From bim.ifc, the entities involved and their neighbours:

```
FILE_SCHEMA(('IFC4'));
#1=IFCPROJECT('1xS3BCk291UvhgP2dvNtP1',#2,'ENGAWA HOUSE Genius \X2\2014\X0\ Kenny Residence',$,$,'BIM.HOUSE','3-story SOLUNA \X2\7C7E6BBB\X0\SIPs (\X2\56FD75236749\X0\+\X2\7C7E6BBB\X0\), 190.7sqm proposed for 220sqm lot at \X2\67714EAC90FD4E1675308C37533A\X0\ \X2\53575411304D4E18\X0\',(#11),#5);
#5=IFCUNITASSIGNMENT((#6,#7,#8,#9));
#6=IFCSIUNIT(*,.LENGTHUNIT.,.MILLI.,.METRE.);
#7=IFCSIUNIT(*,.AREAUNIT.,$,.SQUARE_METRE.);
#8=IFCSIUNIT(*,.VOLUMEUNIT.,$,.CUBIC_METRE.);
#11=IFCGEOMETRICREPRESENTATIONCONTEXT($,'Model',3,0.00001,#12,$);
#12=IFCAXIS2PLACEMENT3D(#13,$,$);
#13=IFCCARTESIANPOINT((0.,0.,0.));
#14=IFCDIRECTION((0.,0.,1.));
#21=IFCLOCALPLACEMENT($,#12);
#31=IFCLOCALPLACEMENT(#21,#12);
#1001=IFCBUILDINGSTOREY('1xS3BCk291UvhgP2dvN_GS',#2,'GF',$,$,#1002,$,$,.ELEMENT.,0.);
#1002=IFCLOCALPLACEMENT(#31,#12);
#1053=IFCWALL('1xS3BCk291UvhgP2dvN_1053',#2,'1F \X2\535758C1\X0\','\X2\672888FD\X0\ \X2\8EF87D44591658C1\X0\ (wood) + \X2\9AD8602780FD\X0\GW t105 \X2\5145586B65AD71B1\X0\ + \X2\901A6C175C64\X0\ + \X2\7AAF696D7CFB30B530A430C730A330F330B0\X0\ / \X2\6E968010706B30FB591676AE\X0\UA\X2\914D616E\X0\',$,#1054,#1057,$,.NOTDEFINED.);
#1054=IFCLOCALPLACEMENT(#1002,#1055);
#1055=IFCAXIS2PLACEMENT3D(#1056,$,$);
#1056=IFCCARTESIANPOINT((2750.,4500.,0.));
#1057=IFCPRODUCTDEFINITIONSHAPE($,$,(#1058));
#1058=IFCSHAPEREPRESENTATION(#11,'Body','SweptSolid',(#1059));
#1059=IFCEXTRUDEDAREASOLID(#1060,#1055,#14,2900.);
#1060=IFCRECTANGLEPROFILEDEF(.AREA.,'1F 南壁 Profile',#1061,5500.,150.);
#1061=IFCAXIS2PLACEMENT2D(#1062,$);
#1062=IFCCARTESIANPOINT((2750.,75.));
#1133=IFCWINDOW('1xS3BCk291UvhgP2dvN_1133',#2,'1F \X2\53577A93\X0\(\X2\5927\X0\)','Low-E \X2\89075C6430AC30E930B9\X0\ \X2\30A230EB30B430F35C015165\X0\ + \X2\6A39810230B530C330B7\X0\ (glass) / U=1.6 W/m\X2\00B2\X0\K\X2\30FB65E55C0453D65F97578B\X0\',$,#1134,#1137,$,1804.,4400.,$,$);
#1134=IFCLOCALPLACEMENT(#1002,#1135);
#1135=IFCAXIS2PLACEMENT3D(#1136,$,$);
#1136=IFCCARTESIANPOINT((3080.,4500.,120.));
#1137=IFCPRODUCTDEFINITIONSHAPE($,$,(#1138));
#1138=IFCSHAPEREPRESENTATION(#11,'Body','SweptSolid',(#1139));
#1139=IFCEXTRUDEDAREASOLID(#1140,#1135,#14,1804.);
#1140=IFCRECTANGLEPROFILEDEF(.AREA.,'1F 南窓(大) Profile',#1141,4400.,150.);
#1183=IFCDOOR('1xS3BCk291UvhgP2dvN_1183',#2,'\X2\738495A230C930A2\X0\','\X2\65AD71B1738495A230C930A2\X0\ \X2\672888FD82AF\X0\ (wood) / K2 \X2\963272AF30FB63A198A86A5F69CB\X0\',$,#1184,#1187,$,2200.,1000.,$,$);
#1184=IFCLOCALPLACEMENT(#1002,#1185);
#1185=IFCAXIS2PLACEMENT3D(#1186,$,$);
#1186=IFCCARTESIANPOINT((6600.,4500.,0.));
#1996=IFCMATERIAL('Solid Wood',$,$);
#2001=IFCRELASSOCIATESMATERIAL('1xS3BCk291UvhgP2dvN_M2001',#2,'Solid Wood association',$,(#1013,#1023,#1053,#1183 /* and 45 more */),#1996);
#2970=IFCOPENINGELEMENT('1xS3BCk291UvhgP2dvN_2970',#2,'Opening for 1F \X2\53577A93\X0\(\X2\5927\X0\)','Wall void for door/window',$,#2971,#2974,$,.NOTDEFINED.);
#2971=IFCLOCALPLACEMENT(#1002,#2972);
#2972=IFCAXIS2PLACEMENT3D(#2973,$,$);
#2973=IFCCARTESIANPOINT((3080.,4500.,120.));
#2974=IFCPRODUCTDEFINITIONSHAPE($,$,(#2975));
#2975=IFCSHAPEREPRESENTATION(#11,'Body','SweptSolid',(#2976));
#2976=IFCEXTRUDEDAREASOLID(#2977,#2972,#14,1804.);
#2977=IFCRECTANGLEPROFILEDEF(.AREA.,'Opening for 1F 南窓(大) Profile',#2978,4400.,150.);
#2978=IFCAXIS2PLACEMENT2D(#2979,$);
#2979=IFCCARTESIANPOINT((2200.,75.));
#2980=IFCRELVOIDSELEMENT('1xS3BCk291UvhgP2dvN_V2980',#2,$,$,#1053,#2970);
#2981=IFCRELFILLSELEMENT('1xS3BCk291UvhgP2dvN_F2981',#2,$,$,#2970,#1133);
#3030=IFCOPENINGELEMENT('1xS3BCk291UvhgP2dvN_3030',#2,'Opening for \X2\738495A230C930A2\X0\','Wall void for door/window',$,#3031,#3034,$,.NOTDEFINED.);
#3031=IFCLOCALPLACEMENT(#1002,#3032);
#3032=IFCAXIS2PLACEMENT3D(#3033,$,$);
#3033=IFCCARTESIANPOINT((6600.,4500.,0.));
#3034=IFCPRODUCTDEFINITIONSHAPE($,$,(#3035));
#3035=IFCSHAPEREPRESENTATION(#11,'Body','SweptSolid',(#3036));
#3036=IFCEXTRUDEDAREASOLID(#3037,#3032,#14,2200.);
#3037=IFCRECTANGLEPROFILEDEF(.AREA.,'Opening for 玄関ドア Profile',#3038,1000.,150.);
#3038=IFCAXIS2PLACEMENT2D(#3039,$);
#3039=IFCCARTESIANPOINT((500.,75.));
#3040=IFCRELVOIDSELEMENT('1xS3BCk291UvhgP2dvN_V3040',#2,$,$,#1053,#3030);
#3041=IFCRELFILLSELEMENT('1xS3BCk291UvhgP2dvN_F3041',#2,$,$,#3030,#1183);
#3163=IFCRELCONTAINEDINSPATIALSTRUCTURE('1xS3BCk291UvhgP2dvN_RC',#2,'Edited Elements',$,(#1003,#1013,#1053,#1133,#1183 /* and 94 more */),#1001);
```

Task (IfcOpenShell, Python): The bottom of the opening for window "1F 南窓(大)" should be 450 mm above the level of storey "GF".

```python
import numpy as np
import ifcopenshell
import ifcopenshell.api.geometry
import ifcopenshell.geom
import ifcopenshell.util.element
import ifcopenshell.util.placement
import ifcopenshell.util.shape
import ifcopenshell.util.unit

model = ifcopenshell.open("bim.ifc")
unit_scale = ifcopenshell.util.unit.calculate_unit_scale(model)

window = model.by_guid("1xS3BCk291UvhgP2dvN_1133")
opening = window.FillsVoids[0].RelatingOpeningElement
storey = ifcopenshell.util.element.get_container(window, ifc_class="IfcBuildingStorey")
level = ifcopenshell.util.placement.get_local_placement(storey.ObjectPlacement)[2, 3]

# The opening's origin need not be at the sill, so measure its lowest point.
shape = ifcopenshell.geom.create_shape(ifcopenshell.geom.settings(), opening)
bottom = ifcopenshell.util.shape.get_shape_bottom_elevation(shape, shape.geometry) / unit_scale
dz = level + 0.45 / unit_scale - bottom

shift = np.array([0.0, 0.0, dz])
# The window is not placed relative to its opening, so move both.
for product in (opening, window):
    matrix = ifcopenshell.util.placement.get_local_placement(product.ObjectPlacement)
    matrix[:3, 3] += shift
    ifcopenshell.api.geometry.edit_object_placement(model, product=product, matrix=matrix, is_si=False)

print(f"moved by {dz * unit_scale:+.3f} m")

model.write("bim-out.ifc")
```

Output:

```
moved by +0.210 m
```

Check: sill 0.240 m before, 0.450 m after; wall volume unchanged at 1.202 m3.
